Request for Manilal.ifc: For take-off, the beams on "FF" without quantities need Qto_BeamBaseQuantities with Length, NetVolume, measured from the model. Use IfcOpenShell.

First a look at what the model holds.

```python
import ifcopenshell
import ifcopenshell.util.element
import ifcopenshell.util.unit

model = ifcopenshell.open("Manilal.ifc")
print(model.schema)
for unit_type in ("LENGTHUNIT", "AREAUNIT", "VOLUMEUNIT"):
    print(unit_type, ifcopenshell.util.unit.calculate_unit_scale(model, unit_type))
storey = next(s for s in model.by_type("IfcBuildingStorey") if s.Name == "FF")
beams = [e for e in ifcopenshell.util.element.get_decomposition(storey) if e.is_a("IfcBeam")]
for e in sorted(beams, key=lambda e: e.id()):
    print(e.id(), e.is_a(), e.Name, list(ifcopenshell.util.element.get_psets(e, qtos_only=True)), sep=" | ")
```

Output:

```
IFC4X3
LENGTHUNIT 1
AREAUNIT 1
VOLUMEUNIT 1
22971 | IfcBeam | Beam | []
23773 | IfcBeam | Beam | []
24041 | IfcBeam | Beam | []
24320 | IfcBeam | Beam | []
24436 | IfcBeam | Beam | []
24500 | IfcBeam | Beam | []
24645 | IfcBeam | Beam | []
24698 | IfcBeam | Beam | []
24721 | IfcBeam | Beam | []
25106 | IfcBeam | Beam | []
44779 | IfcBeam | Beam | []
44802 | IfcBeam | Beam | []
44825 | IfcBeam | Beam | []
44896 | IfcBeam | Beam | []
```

```python
import ifcopenshell
import ifcopenshell.api.pset
import ifcopenshell.geom
import ifcopenshell.util.element
import ifcopenshell.util.shape
import ifcopenshell.util.unit

model = ifcopenshell.open("Manilal.ifc")
unit_scale = ifcopenshell.util.unit.calculate_unit_scale(model)
volume_scale = ifcopenshell.util.unit.calculate_unit_scale(model, "VOLUMEUNIT")
settings = ifcopenshell.geom.settings()

storey = next(s for s in model.by_type("IfcBuildingStorey") if s.Name == "FF")
beams = [e for e in ifcopenshell.util.element.get_decomposition(storey) if e.is_a("IfcBeam")]

for e in sorted(beams, key=lambda e: e.id()):
    if ifcopenshell.util.element.get_psets(e, qtos_only=True, should_inherit=False):
        continue
    # Geometry comes back in metres, in the element's own axes.
    shape = ifcopenshell.geom.create_shape(settings, e)
    values = {
        "Length": ifcopenshell.util.shape.get_max_xyz(shape.geometry) / unit_scale,
        "NetVolume": ifcopenshell.util.shape.get_volume(shape.geometry) / volume_scale,
    }
    qto = ifcopenshell.api.pset.add_qto(model, product=e, name="Qto_BeamBaseQuantities")
    ifcopenshell.api.pset.edit_qto(model, qto=qto, properties=values)
    print(e.id(), {k: round(v, 3) for k, v in values.items()})

model.write("Manilal_updated.ifc")
```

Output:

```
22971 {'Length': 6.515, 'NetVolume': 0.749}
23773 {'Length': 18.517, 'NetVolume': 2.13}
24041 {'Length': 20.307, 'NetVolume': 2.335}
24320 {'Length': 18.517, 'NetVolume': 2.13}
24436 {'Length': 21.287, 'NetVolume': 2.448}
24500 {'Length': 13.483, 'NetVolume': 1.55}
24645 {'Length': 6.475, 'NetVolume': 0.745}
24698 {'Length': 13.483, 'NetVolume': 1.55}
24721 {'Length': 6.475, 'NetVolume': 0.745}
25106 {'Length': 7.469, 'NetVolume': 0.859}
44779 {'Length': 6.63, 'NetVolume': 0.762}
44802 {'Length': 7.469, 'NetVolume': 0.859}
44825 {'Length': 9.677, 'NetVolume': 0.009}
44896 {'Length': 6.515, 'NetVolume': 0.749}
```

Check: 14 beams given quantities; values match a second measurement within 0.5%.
